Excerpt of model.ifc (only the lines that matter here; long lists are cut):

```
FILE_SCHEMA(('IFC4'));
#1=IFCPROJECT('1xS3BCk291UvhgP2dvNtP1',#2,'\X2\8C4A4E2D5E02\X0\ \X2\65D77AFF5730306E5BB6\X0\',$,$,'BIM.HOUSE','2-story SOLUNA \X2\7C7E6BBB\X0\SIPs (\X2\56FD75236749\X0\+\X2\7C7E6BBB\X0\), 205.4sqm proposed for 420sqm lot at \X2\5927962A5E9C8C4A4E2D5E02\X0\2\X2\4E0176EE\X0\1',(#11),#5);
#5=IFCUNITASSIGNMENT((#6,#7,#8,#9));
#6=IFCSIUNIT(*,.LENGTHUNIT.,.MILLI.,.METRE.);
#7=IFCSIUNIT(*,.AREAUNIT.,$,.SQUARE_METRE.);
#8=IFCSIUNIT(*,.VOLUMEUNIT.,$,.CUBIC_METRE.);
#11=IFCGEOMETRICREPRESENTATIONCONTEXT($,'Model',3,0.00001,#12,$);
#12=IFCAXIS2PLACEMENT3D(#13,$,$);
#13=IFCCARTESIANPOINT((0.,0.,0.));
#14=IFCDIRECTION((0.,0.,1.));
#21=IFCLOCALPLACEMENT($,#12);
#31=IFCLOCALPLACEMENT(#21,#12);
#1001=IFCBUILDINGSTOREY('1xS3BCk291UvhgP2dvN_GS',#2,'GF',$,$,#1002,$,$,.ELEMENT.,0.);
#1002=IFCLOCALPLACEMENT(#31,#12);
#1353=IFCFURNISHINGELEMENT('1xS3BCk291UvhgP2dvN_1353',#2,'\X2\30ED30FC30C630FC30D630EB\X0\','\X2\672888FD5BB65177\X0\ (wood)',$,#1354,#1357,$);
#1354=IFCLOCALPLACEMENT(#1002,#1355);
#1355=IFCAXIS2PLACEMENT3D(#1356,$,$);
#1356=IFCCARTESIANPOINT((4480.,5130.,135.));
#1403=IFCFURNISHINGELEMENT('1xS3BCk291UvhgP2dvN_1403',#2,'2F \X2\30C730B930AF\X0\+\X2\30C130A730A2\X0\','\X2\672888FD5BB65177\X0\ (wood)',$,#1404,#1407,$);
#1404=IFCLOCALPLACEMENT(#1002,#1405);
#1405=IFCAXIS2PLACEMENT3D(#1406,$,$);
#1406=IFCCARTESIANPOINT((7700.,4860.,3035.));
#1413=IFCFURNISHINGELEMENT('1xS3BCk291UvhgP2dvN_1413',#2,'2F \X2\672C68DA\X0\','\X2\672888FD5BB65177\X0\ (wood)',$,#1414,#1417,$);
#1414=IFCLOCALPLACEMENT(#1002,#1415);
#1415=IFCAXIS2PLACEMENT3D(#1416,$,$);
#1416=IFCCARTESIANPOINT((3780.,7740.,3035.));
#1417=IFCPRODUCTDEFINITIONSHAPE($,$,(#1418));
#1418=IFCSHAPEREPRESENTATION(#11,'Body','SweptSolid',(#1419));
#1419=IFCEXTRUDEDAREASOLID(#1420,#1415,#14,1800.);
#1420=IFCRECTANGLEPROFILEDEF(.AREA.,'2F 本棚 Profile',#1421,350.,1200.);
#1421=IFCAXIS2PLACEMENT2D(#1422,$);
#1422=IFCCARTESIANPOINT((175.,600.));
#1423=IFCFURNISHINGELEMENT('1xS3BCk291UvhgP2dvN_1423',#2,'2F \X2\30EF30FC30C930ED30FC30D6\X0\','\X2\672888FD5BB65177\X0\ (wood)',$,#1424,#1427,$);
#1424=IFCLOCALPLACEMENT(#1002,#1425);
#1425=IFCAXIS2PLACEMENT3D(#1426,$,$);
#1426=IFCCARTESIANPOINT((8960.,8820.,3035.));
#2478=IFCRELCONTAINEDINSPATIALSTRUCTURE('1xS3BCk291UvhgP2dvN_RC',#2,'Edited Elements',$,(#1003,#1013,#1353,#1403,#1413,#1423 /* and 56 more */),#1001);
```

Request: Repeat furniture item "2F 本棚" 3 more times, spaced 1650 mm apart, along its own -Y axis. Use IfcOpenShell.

```python
import ifcopenshell
import ifcopenshell.api.geometry
import ifcopenshell.api.root
import ifcopenshell.util.element
import ifcopenshell.util.placement
import ifcopenshell.util.unit

model = ifcopenshell.open("model.ifc")
unit_scale = ifcopenshell.util.unit.calculate_unit_scale(model)


def reuse_history(source, copy):
    """copy_class also copies each property set's owner history, people and application; keep the originals."""
    for rel in copy.IsDefinedBy:
        if rel.is_a("IfcRelDefinesByProperties") and (history := rel.RelatingPropertyDefinition.OwnerHistory):
            rel.RelatingPropertyDefinition.OwnerHistory = source.OwnerHistory
            ifcopenshell.util.element.remove_deep2(model, history)


source = model.by_guid("1xS3BCk291UvhgP2dvN_1413")
base = ifcopenshell.util.placement.get_local_placement(source.ObjectPlacement)
step = -base[:3, 1] * 1.65 / unit_scale

for i in range(1, 4):
    copy = ifcopenshell.api.root.copy_class(model, product=source)
    copy.Representation = ifcopenshell.util.element.copy_deep(
        model, source.Representation, exclude=["IfcGeometricRepresentationContext", "IfcRepresentationMap"]
    )
    reuse_history(source, copy)
    matrix = base.copy()
    matrix[:3, 3] += i * step
    print("added at", matrix[:3, 3].round(3) + 0.0)
    ifcopenshell.api.geometry.edit_object_placement(model, product=copy, matrix=matrix, is_si=False)

model.write("model_rev.ifc")
```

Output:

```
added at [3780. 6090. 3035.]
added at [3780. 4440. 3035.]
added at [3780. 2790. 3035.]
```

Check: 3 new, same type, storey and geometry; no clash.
